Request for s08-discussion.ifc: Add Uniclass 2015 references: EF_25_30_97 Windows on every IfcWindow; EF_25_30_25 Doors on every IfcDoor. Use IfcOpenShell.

First a look at what the model holds.

```python
import ifcopenshell

model = ifcopenshell.open("s08-discussion.ifc")
print(model.schema)
print("classifications:", [c.Name for c in model.by_type("IfcClassification")])
for ifc_class in ("IfcDoor", "IfcRoof", "IfcStair", "IfcWall", "IfcWindow"):
    print(ifc_class, len(model.by_type(ifc_class)))
```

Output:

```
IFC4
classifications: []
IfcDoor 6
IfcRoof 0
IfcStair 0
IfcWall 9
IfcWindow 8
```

```python
import ifcopenshell
import ifcopenshell.api.classification

model = ifcopenshell.open("s08-discussion.ifc")

system = ifcopenshell.api.classification.add_classification(model, classification="Uniclass 2015")

codes = {
    "IfcWindow": ("EF_25_30_97", "Windows"),
    "IfcDoor": ("EF_25_30_25", "Doors"),
}
for ifc_class, (code, name) in codes.items():
    products = model.by_type(ifc_class)
    ifcopenshell.api.classification.add_reference(
        model, products=products, classification=system, identification=code, name=name
    )
    print(code, len(products))

model.write("s08-discussion_v2.ifc")
```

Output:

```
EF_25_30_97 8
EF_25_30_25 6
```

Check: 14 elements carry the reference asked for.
